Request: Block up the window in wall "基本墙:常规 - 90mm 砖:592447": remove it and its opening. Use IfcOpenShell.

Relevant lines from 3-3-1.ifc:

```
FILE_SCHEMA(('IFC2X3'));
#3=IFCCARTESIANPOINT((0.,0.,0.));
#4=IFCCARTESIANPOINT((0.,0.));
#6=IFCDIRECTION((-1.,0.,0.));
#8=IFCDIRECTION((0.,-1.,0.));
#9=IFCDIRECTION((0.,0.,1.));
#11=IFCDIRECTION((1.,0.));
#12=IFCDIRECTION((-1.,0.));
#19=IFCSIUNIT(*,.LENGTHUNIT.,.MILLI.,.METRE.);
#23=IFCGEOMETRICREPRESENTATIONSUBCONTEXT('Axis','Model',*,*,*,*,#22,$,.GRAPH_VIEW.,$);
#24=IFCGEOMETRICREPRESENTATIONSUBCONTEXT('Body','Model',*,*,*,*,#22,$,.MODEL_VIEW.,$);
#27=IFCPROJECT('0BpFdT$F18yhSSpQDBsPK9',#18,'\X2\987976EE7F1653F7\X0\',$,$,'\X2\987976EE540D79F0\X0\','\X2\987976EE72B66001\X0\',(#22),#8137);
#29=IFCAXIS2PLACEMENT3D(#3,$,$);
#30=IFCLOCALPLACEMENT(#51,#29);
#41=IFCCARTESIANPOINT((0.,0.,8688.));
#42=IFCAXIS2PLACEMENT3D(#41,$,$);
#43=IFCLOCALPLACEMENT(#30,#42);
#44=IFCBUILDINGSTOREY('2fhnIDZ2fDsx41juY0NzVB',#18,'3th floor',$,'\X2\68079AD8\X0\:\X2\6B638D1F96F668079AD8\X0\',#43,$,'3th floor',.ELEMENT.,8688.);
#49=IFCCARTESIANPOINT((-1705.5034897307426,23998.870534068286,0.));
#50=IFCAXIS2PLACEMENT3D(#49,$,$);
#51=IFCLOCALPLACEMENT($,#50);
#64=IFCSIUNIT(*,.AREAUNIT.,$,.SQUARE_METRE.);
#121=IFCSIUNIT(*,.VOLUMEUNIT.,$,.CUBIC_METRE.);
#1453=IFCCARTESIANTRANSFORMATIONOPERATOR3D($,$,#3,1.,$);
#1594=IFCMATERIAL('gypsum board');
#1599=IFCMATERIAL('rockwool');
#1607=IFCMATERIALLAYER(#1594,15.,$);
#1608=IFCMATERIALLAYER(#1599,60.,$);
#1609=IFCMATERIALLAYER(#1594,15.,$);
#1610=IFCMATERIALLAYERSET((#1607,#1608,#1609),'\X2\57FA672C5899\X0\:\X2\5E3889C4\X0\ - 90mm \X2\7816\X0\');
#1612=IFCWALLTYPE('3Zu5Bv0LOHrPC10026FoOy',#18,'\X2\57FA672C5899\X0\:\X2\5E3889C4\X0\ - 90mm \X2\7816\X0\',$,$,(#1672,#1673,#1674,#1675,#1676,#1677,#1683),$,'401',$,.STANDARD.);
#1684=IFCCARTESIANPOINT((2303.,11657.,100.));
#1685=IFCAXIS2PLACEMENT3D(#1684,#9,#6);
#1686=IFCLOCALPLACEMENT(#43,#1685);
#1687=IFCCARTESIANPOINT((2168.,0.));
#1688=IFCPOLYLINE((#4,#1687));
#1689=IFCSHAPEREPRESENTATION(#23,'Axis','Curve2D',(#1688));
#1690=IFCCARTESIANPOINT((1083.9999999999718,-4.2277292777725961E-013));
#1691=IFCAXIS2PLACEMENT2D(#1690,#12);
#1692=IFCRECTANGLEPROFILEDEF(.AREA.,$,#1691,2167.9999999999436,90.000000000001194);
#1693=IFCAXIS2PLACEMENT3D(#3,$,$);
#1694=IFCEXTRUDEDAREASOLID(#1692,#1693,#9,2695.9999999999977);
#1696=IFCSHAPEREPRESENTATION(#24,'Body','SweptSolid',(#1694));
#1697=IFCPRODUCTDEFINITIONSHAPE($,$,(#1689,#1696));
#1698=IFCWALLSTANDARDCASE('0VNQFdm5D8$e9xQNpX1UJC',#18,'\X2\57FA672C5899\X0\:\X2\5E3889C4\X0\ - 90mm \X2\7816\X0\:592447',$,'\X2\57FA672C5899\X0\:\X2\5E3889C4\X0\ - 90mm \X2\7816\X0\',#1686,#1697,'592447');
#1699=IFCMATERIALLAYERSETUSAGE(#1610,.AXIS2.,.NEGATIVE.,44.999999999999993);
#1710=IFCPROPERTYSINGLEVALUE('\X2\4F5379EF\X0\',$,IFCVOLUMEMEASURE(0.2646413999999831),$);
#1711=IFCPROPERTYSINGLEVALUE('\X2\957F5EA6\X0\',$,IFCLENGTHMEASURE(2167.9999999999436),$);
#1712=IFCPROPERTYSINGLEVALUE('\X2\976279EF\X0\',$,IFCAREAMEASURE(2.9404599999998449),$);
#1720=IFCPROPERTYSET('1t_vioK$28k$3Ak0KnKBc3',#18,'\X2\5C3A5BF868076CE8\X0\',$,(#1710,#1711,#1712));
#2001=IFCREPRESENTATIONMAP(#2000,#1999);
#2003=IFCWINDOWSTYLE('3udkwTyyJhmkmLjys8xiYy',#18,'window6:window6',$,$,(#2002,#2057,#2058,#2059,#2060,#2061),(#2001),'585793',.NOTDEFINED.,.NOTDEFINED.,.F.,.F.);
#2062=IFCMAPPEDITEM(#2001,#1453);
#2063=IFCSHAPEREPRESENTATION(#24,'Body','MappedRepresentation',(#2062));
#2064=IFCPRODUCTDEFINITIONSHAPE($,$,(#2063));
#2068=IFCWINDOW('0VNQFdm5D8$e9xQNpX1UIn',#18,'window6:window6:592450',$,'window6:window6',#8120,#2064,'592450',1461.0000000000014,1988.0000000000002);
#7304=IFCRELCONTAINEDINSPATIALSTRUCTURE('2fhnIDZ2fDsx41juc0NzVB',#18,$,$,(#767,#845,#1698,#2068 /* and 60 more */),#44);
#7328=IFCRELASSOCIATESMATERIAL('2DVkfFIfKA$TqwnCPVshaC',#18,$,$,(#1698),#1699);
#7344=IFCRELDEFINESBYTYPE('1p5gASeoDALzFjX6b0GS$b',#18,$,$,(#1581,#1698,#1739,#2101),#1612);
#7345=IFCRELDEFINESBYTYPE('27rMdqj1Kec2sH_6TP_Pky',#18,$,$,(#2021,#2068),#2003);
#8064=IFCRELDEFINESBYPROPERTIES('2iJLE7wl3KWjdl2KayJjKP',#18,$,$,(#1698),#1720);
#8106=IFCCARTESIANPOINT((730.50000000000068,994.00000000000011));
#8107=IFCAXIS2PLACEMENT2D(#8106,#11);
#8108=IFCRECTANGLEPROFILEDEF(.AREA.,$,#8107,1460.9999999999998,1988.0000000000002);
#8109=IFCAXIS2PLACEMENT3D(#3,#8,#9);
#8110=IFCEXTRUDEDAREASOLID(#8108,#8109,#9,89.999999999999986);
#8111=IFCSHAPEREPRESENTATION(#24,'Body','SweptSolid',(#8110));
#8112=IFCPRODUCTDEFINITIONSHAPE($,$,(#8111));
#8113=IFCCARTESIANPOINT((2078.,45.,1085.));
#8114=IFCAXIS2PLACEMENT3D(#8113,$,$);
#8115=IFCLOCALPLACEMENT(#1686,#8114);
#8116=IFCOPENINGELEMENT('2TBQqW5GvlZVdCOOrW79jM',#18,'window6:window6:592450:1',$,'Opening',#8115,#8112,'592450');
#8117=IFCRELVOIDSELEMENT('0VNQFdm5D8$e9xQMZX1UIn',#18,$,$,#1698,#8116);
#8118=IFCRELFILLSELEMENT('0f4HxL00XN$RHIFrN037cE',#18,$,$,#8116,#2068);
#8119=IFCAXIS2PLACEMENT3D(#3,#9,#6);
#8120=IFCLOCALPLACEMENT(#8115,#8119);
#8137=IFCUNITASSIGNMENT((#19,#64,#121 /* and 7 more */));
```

```python
import ifcopenshell
import ifcopenshell.api.feature
import ifcopenshell.api.pset
import ifcopenshell.api.root
import ifcopenshell.geom
import ifcopenshell.util.element
import ifcopenshell.util.shape
import ifcopenshell.util.unit

model = ifcopenshell.open("3-3-1.ifc")
area_scale = ifcopenshell.util.unit.calculate_unit_scale(model, "AREAUNIT")
volume_scale = ifcopenshell.util.unit.calculate_unit_scale(model, "VOLUMEUNIT")
settings = ifcopenshell.geom.settings()


def volume(element):
    """Net volume in cubic metres, openings subtracted."""
    shape = ifcopenshell.geom.create_shape(settings, element)
    return ifcopenshell.util.shape.get_volume(shape.geometry)


window = model.by_guid("0VNQFdm5D8$e9xQNpX1UIn")
opening = window.FillsVoids[0].RelatingOpeningElement
wall = opening.VoidsElements[0].RelatingBuildingElement
before = volume(wall)

ifcopenshell.api.root.remove_product(model, product=window)
ifcopenshell.api.feature.remove_feature(model, feature=opening)

after = volume(wall)
thickness = 0.09  # wall thickness in metres

# Update the wall's stored quantities.
pset = model.by_id(ifcopenshell.util.element.get_pset(wall, "尺寸标注", should_inherit=False)["id"])
ifcopenshell.api.pset.edit_pset(model, pset=pset, properties={
    "体积": model.create_entity("IfcVolumeMeasure", after / volume_scale),
    "面积": model.create_entity("IfcAreaMeasure", after / thickness / area_scale),
})

print(f"wall volume {before:.3f} -> {after:.3f} m3")

model.write("3-3-1_updated.ifc")
```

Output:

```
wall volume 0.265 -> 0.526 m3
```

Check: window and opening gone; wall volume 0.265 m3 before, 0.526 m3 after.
